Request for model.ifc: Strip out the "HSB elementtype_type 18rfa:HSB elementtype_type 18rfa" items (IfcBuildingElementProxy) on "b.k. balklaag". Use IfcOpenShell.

First a look at what the model holds.

```python
import ifcopenshell
import ifcopenshell.util.element

model = ifcopenshell.open("model.ifc")
print(model.schema)
storey = next(s for s in model.by_type("IfcBuildingStorey") if s.Name == "b.k. balklaag")
proxies = [e for e in ifcopenshell.util.element.get_decomposition(storey) if e.is_a("IfcBuildingElementProxy")]
seen = {}
for e in proxies:
    element_type = ifcopenshell.util.element.get_type(e)
    name = element_type.Name if element_type not in (None, e) else None
    seen[name] = seen.get(name, 0) + 1
for name, count in sorted(seen.items(), key=str):
    print(count, "x", name)
```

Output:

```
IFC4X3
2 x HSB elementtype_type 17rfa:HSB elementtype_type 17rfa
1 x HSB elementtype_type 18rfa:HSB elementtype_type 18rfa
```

```python
import ifcopenshell
import ifcopenshell.api.root
import ifcopenshell.util.element

model = ifcopenshell.open("model.ifc")

storey = next(s for s in model.by_type("IfcBuildingStorey") if s.Name == "b.k. balklaag")
proxies = [e for e in ifcopenshell.util.element.get_decomposition(storey) if e.is_a("IfcBuildingElementProxy")]
targets = [e for e in proxies if (t := ifcopenshell.util.element.get_type(e)) not in (None, e) and t.Name == "HSB elementtype_type 18rfa:HSB elementtype_type 18rfa"]

for e in targets:
    ifcopenshell.api.root.remove_product(model, product=e)
print(len(targets), "removed")

model.write("model_v2.ifc")
```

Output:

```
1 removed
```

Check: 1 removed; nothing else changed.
